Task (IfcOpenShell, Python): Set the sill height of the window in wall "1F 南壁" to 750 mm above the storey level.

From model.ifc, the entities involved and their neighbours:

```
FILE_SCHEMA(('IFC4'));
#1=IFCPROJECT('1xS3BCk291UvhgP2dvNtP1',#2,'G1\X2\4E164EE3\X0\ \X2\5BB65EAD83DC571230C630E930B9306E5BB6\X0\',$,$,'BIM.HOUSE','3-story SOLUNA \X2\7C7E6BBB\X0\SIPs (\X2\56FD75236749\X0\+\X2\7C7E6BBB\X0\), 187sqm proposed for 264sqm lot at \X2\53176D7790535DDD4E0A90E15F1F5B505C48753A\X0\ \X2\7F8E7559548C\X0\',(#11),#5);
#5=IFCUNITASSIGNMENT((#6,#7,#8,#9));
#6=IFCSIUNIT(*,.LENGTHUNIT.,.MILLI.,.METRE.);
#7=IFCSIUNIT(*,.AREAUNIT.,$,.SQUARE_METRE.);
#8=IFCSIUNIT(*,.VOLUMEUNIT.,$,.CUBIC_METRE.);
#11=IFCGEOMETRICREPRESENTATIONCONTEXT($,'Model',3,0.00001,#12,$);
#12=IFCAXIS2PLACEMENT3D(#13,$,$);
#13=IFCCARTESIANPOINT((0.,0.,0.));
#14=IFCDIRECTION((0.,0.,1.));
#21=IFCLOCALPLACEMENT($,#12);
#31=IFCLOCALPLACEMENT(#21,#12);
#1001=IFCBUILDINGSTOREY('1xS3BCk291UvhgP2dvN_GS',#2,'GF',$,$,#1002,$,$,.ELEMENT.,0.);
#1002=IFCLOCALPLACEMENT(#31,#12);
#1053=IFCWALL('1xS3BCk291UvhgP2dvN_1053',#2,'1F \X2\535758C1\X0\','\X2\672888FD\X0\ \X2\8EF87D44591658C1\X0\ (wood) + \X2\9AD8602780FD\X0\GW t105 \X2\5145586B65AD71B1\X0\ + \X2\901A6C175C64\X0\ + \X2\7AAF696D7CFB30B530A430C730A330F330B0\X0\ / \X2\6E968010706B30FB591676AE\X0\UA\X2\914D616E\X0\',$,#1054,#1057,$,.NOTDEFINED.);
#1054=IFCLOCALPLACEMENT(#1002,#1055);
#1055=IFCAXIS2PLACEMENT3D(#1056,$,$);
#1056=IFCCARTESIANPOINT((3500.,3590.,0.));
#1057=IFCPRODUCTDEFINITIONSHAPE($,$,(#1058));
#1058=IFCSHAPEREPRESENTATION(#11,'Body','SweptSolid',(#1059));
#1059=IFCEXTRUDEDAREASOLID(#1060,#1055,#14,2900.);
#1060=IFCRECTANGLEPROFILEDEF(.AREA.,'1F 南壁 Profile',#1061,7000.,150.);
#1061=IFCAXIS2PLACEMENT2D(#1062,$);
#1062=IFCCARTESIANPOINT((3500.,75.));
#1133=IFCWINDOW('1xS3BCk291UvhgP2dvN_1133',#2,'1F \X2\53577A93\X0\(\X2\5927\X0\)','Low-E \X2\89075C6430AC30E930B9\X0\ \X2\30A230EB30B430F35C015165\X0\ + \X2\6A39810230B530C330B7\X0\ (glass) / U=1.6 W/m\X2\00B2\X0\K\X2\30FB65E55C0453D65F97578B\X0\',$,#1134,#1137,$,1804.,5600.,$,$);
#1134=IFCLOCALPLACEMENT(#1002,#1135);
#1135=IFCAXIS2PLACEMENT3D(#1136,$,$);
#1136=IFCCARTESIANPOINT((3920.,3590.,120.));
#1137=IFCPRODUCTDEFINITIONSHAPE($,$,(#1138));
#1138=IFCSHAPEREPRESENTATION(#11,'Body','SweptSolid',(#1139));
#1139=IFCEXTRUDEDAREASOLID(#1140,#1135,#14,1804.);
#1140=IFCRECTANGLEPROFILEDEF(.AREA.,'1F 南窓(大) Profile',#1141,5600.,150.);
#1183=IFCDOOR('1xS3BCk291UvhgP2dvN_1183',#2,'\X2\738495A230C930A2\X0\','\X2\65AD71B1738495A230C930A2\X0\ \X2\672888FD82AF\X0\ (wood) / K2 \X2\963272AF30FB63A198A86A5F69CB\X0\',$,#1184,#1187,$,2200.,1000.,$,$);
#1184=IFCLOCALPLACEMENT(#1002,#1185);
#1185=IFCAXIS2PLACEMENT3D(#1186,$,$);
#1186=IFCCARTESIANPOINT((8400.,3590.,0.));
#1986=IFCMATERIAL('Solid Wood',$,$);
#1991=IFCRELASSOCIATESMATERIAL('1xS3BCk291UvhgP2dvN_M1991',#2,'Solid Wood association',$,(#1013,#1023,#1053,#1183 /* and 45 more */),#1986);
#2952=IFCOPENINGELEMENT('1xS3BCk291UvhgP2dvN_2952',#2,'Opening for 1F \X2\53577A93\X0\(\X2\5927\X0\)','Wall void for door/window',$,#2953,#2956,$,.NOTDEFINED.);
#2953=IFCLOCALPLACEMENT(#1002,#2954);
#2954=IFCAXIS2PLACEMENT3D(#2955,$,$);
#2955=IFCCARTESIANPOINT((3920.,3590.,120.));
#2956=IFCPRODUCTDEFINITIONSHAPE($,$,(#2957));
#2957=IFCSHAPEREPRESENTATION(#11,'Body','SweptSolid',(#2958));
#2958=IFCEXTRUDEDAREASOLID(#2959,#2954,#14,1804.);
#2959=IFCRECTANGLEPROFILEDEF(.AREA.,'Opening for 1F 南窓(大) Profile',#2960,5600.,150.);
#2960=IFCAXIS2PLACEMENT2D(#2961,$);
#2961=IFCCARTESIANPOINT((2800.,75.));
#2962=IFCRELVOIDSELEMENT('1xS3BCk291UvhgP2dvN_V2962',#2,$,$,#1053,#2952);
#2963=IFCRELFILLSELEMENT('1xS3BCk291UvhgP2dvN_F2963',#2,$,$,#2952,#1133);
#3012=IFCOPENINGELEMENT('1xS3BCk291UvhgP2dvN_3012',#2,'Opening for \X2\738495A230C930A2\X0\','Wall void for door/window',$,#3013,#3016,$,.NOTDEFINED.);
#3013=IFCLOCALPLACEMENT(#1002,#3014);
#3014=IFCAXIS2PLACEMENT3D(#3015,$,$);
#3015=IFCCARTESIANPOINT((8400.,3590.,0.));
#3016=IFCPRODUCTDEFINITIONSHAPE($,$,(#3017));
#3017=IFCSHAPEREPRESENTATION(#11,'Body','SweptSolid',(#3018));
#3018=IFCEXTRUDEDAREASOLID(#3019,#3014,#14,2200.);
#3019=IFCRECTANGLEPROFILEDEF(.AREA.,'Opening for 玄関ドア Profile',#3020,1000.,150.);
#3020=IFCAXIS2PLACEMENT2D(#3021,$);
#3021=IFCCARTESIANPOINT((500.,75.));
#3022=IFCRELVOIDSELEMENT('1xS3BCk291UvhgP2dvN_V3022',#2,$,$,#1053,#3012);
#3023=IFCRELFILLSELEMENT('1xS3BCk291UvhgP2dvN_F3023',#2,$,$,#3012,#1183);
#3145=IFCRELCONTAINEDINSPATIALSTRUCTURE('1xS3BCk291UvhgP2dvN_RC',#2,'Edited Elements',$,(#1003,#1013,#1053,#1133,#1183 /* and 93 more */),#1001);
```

```python
import numpy as np
import ifcopenshell
import ifcopenshell.api.geometry
import ifcopenshell.geom
import ifcopenshell.util.element
import ifcopenshell.util.placement
import ifcopenshell.util.shape
import ifcopenshell.util.unit

model = ifcopenshell.open("model.ifc")
unit_scale = ifcopenshell.util.unit.calculate_unit_scale(model)

window = model.by_guid("1xS3BCk291UvhgP2dvN_1133")
opening = window.FillsVoids[0].RelatingOpeningElement
storey = ifcopenshell.util.element.get_container(window, ifc_class="IfcBuildingStorey")
level = ifcopenshell.util.placement.get_local_placement(storey.ObjectPlacement)[2, 3]

# The opening's origin need not be at the sill, so measure its lowest point.
shape = ifcopenshell.geom.create_shape(ifcopenshell.geom.settings(), opening)
bottom = ifcopenshell.util.shape.get_shape_bottom_elevation(shape, shape.geometry) / unit_scale
dz = level + 0.75 / unit_scale - bottom

shift = np.array([0.0, 0.0, dz])
# The window is not placed relative to its opening, so move both.
for product in (opening, window):
    matrix = ifcopenshell.util.placement.get_local_placement(product.ObjectPlacement)
    matrix[:3, 3] += shift
    ifcopenshell.api.geometry.edit_object_placement(model, product=product, matrix=matrix, is_si=False)

print(f"moved by {dz * unit_scale:+.3f} m")

model.write("model-out.ifc")
```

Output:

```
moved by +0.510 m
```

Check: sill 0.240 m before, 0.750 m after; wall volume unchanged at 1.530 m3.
